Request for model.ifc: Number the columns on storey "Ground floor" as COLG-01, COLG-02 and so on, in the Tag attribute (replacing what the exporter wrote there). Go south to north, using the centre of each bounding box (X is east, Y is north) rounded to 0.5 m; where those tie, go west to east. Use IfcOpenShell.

First a look at what the model holds.

```python
import ifcopenshell
import ifcopenshell.util.element
import ifcopenshell.util.placement

model = ifcopenshell.open("model.ifc")
print(model.schema)
storey = next(s for s in model.by_type("IfcBuildingStorey") if s.Name == "Ground floor")
columns = [e for e in ifcopenshell.util.element.get_decomposition(storey) if e.is_a("IfcColumn")]
for e in sorted(columns, key=lambda e: e.id()):
    origin = ifcopenshell.util.placement.get_local_placement(e.ObjectPlacement)[:3, 3]
    print(e.id(), e.Tag, e.Name, origin.round(2) + 0.0, sep=" | ")
```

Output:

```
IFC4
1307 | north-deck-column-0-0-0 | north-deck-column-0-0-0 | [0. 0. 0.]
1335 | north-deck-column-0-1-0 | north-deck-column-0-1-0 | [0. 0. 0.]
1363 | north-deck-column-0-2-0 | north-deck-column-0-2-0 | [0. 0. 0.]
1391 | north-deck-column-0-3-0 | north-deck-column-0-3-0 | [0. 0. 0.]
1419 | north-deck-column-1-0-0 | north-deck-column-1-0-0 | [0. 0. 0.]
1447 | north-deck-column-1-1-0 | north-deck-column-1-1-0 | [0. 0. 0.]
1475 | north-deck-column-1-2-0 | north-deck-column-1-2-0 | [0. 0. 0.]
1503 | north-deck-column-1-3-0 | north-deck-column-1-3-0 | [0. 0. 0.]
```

```python
import ifcopenshell
import ifcopenshell.geom
import ifcopenshell.util.element
import ifcopenshell.util.shape

model = ifcopenshell.open("model.ifc")
settings = ifcopenshell.geom.settings()
settings.set("use-world-coords", True)


def centre(element):
    shape = ifcopenshell.geom.create_shape(settings, element)
    return ifcopenshell.util.shape.get_bbox_centroid(shape.geometry)


storey = next(s for s in model.by_type("IfcBuildingStorey") if s.Name == "Ground floor")
columns = [e for e in ifcopenshell.util.element.get_decomposition(storey) if e.is_a("IfcColumn")]

# Insertion points can sit at a corner or the storey origin, so sort by the geometry (in metres).
centres = {e: centre(e) for e in columns}
columns.sort(key=lambda e: (round(centres[e][1] / 0.5), centres[e][0]))

for i, e in enumerate(columns, start=1):
    number = f"COLG-{i:02d}"
    e.Tag = number
    print(e.id(), number)

model.write("model_v2.ifc")
```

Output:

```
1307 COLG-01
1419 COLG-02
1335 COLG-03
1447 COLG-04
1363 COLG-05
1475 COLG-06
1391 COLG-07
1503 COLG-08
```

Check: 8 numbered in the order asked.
